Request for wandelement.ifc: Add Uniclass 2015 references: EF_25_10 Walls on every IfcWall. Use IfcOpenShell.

First a look at what the model holds.

```python
import ifcopenshell

model = ifcopenshell.open("wandelement.ifc")
print(model.schema)
print("classifications:", [c.Name for c in model.by_type("IfcClassification")])
for ifc_class in ("IfcDoor", "IfcRoof", "IfcStair", "IfcWall", "IfcWindow"):
    print(ifc_class, len(model.by_type(ifc_class)))
```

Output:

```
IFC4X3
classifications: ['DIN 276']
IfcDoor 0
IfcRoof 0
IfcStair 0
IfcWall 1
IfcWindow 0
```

```python
import ifcopenshell
import ifcopenshell.api.classification

model = ifcopenshell.open("wandelement.ifc")

system = ifcopenshell.api.classification.add_classification(model, classification="Uniclass 2015")

codes = {
    "IfcWall": ("EF_25_10", "Walls"),
}
for ifc_class, (code, name) in codes.items():
    products = model.by_type(ifc_class)
    ifcopenshell.api.classification.add_reference(
        model, products=products, classification=system, identification=code, name=name
    )
    print(code, len(products))

model.write("wandelement-out.ifc")
```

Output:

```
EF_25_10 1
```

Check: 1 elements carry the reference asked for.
